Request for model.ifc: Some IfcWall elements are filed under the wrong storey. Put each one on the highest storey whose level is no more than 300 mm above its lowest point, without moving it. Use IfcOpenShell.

First a look at what the model holds.

```python
import ifcopenshell
import ifcopenshell.util.element
import ifcopenshell.util.placement

model = ifcopenshell.open("model.ifc")
print(model.schema)
for storey in model.by_type("IfcBuildingStorey"):
    level = ifcopenshell.util.placement.get_storey_elevation(storey)
    count = sum(e.is_a("IfcWall") for e in ifcopenshell.util.element.get_contained(storey))
    print(storey.id(), storey.Name, round(level, 3), count, sep=" | ")
```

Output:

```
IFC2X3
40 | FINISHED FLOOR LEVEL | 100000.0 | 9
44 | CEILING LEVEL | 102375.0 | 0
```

```python
import ifcopenshell
import ifcopenshell.api.spatial
import ifcopenshell.geom
import ifcopenshell.util.element
import ifcopenshell.util.placement
import ifcopenshell.util.shape
import ifcopenshell.util.unit

model = ifcopenshell.open("model.ifc")
unit_scale = ifcopenshell.util.unit.calculate_unit_scale(model)
settings = ifcopenshell.geom.settings()

levels = sorted(
    ((ifcopenshell.util.placement.get_storey_elevation(s) * unit_scale, s) for s in model.by_type("IfcBuildingStorey")),
    key=lambda pair: pair[0],
)

for e in model.by_type("IfcWall"):
    current = e.ContainedInStructure[0].RelatingStructure if e.ContainedInStructure else None
    if current is None or not current.is_a("IfcBuildingStorey"):
        continue
    shape = ifcopenshell.geom.create_shape(settings, e)
    bottom = ifcopenshell.util.shape.get_shape_bottom_elevation(shape, shape.geometry)
    below = [s for level, s in levels if level <= bottom + 0.3]
    storey = below[-1] if below else levels[0][1]
    if storey != current:
        # assign_container keeps the world position.
        ifcopenshell.api.spatial.assign_container(model, products=[e], relating_structure=storey)
        print(e.id(), current.Name, "->", storey.Name)

model.write("model_v2.ifc")
```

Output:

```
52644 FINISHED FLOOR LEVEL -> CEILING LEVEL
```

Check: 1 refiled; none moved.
